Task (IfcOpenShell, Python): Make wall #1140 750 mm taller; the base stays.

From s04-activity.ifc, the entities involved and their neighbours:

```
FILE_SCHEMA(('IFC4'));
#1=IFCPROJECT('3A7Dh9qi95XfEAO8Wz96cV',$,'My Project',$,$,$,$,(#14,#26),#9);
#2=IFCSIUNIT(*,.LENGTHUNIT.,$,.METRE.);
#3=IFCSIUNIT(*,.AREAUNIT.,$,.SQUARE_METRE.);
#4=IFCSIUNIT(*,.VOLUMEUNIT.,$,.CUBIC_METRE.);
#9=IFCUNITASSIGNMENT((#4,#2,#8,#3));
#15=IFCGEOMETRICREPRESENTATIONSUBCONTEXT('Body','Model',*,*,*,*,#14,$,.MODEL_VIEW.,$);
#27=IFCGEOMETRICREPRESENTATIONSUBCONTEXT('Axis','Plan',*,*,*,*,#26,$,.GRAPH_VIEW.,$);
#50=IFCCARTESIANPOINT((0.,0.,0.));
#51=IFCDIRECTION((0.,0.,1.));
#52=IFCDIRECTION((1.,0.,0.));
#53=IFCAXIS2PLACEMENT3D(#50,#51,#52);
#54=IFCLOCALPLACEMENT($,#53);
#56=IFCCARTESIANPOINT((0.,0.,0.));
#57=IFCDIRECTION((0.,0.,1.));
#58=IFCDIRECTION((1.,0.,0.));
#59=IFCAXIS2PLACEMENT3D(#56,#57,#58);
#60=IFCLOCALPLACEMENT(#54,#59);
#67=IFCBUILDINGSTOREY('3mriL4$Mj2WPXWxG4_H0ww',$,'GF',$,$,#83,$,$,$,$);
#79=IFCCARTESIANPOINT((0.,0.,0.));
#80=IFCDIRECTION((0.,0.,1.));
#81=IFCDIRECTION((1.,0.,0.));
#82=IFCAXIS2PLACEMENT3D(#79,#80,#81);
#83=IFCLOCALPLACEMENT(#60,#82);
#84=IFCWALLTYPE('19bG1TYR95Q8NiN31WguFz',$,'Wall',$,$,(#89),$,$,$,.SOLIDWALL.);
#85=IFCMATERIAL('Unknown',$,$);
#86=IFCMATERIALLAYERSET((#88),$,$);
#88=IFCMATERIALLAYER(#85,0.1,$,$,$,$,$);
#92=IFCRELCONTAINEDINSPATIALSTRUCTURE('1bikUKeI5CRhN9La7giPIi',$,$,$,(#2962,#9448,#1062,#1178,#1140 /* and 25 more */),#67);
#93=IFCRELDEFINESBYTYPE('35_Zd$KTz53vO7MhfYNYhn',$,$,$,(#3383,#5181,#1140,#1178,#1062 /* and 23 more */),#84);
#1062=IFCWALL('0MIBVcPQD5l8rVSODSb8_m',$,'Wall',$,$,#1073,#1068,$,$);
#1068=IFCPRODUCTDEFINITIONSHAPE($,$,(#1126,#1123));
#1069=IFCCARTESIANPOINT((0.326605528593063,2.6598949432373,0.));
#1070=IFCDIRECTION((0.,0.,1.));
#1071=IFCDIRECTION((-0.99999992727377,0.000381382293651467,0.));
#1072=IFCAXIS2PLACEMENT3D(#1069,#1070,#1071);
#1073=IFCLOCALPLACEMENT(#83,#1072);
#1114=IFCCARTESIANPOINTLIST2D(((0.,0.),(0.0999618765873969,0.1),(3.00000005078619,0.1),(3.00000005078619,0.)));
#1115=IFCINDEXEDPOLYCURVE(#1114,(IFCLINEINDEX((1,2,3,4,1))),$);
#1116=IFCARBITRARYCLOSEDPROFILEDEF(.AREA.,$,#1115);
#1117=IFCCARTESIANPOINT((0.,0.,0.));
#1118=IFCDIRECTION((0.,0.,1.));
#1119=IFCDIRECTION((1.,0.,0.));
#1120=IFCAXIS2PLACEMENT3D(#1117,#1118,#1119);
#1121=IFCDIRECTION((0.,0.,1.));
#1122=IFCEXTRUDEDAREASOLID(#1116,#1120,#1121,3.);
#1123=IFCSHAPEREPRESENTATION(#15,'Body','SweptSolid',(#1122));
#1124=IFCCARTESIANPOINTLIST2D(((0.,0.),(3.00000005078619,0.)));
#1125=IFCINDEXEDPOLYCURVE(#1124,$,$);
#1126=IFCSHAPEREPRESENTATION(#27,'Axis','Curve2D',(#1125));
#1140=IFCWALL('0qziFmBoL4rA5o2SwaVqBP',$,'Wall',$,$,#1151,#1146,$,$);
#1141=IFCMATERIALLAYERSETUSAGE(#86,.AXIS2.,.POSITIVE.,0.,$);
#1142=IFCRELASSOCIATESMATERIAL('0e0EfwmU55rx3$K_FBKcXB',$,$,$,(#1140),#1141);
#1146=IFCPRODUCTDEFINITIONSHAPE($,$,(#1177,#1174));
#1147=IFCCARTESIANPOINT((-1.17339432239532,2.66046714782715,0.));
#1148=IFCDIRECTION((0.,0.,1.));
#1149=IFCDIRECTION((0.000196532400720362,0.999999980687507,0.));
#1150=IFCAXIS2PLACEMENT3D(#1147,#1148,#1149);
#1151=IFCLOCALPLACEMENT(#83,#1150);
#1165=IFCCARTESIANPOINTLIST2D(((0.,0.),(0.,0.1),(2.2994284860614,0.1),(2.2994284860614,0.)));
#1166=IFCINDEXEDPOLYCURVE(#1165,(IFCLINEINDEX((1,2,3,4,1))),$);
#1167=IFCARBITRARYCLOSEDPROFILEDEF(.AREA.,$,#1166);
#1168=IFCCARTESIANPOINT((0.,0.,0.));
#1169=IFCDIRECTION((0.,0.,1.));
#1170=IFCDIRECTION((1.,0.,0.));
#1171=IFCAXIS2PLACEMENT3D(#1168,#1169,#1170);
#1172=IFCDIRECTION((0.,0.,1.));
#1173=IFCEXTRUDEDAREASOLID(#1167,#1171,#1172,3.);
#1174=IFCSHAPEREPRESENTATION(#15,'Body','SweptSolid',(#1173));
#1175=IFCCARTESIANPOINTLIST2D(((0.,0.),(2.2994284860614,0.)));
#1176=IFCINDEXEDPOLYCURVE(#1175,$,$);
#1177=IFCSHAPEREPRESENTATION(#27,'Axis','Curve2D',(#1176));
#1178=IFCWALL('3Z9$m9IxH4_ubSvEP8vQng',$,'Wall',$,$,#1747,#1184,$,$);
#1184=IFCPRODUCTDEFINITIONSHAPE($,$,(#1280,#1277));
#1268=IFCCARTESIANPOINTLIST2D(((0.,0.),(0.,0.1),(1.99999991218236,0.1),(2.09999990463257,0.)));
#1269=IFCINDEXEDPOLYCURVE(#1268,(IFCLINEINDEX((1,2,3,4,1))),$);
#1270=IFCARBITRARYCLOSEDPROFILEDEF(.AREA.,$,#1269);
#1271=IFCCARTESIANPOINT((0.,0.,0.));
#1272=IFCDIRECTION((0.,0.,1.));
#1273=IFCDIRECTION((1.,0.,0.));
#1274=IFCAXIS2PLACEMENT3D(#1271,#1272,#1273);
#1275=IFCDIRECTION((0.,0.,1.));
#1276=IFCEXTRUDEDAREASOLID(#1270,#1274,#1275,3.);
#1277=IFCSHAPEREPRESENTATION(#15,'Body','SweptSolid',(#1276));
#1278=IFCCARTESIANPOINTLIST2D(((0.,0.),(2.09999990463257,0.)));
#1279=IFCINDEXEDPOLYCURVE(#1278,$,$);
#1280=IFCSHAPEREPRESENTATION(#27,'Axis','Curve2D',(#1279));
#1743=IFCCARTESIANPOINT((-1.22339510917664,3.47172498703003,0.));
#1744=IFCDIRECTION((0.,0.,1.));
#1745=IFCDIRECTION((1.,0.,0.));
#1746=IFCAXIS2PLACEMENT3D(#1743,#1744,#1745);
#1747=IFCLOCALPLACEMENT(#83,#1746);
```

```python
import ifcopenshell
import ifcopenshell.geom
import ifcopenshell.util.representation
import ifcopenshell.util.shape
import ifcopenshell.util.unit

model = ifcopenshell.open("s04-activity.ifc")
unit_scale = ifcopenshell.util.unit.calculate_unit_scale(model)
settings = ifcopenshell.geom.settings()


def volume(element):
    """Net volume in cubic metres, openings subtracted."""
    shape = ifcopenshell.geom.create_shape(settings, element)
    return ifcopenshell.util.shape.get_volume(shape.geometry)


wall = model.by_id(1140)
before = volume(wall)

body = ifcopenshell.util.representation.get_representation(wall, "Model", "Body")
solid = body.Items[0]
old_height = solid.Depth
solid.Depth += 0.75 / unit_scale
after = volume(wall)

print(f"height {old_height:g} -> {solid.Depth:g}, volume {before:.3f} -> {after:.3f} m3")

model.write("s04-activity_rev.ifc")
```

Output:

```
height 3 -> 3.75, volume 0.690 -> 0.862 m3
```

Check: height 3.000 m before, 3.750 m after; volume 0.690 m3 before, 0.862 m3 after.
